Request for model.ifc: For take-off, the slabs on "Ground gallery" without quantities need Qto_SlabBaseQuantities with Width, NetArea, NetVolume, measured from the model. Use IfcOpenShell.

First a look at what the model holds.

```python
import ifcopenshell
import ifcopenshell.util.element
import ifcopenshell.util.unit

model = ifcopenshell.open("model.ifc")
print(model.schema)
for unit_type in ("LENGTHUNIT", "AREAUNIT", "VOLUMEUNIT"):
    print(unit_type, ifcopenshell.util.unit.calculate_unit_scale(model, unit_type))
storey = next(s for s in model.by_type("IfcBuildingStorey") if s.Name == "Ground gallery")
slabs = [e for e in ifcopenshell.util.element.get_decomposition(storey) if e.is_a("IfcSlab")]
for e in sorted(slabs, key=lambda e: e.id()):
    print(e.id(), e.is_a(), e.Name, list(ifcopenshell.util.element.get_psets(e, qtos_only=True)), sep=" | ")
```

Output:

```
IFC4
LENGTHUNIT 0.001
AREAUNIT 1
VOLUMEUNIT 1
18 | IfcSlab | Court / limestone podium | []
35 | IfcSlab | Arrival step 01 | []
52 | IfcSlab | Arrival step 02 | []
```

```python
import ifcopenshell
import ifcopenshell.api.pset
import ifcopenshell.geom
import ifcopenshell.util.element
import ifcopenshell.util.shape
import ifcopenshell.util.unit

model = ifcopenshell.open("model.ifc")
unit_scale = ifcopenshell.util.unit.calculate_unit_scale(model)
area_scale = ifcopenshell.util.unit.calculate_unit_scale(model, "AREAUNIT")
volume_scale = ifcopenshell.util.unit.calculate_unit_scale(model, "VOLUMEUNIT")
settings = ifcopenshell.geom.settings()

storey = next(s for s in model.by_type("IfcBuildingStorey") if s.Name == "Ground gallery")
slabs = [e for e in ifcopenshell.util.element.get_decomposition(storey) if e.is_a("IfcSlab")]

for e in sorted(slabs, key=lambda e: e.id()):
    if ifcopenshell.util.element.get_psets(e, qtos_only=True, should_inherit=False):
        continue
    # Geometry comes back in metres, in the element's own axes.
    shape = ifcopenshell.geom.create_shape(settings, e)
    values = {
        "Width": ifcopenshell.util.shape.get_z(shape.geometry) / unit_scale,
        "NetArea": ifcopenshell.util.shape.get_footprint_area(shape.geometry) / area_scale,
        "NetVolume": ifcopenshell.util.shape.get_volume(shape.geometry) / volume_scale,
    }
    qto = ifcopenshell.api.pset.add_qto(model, product=e, name="Qto_SlabBaseQuantities")
    ifcopenshell.api.pset.edit_qto(model, qto=qto, properties=values)
    print(e.id(), {k: round(v, 3) for k, v in values.items()})

model.write("model_v2.ifc")
```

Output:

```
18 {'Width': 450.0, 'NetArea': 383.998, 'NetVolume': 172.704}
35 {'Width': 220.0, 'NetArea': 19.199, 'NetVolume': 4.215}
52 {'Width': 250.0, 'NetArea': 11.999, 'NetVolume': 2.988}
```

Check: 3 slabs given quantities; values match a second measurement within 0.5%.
